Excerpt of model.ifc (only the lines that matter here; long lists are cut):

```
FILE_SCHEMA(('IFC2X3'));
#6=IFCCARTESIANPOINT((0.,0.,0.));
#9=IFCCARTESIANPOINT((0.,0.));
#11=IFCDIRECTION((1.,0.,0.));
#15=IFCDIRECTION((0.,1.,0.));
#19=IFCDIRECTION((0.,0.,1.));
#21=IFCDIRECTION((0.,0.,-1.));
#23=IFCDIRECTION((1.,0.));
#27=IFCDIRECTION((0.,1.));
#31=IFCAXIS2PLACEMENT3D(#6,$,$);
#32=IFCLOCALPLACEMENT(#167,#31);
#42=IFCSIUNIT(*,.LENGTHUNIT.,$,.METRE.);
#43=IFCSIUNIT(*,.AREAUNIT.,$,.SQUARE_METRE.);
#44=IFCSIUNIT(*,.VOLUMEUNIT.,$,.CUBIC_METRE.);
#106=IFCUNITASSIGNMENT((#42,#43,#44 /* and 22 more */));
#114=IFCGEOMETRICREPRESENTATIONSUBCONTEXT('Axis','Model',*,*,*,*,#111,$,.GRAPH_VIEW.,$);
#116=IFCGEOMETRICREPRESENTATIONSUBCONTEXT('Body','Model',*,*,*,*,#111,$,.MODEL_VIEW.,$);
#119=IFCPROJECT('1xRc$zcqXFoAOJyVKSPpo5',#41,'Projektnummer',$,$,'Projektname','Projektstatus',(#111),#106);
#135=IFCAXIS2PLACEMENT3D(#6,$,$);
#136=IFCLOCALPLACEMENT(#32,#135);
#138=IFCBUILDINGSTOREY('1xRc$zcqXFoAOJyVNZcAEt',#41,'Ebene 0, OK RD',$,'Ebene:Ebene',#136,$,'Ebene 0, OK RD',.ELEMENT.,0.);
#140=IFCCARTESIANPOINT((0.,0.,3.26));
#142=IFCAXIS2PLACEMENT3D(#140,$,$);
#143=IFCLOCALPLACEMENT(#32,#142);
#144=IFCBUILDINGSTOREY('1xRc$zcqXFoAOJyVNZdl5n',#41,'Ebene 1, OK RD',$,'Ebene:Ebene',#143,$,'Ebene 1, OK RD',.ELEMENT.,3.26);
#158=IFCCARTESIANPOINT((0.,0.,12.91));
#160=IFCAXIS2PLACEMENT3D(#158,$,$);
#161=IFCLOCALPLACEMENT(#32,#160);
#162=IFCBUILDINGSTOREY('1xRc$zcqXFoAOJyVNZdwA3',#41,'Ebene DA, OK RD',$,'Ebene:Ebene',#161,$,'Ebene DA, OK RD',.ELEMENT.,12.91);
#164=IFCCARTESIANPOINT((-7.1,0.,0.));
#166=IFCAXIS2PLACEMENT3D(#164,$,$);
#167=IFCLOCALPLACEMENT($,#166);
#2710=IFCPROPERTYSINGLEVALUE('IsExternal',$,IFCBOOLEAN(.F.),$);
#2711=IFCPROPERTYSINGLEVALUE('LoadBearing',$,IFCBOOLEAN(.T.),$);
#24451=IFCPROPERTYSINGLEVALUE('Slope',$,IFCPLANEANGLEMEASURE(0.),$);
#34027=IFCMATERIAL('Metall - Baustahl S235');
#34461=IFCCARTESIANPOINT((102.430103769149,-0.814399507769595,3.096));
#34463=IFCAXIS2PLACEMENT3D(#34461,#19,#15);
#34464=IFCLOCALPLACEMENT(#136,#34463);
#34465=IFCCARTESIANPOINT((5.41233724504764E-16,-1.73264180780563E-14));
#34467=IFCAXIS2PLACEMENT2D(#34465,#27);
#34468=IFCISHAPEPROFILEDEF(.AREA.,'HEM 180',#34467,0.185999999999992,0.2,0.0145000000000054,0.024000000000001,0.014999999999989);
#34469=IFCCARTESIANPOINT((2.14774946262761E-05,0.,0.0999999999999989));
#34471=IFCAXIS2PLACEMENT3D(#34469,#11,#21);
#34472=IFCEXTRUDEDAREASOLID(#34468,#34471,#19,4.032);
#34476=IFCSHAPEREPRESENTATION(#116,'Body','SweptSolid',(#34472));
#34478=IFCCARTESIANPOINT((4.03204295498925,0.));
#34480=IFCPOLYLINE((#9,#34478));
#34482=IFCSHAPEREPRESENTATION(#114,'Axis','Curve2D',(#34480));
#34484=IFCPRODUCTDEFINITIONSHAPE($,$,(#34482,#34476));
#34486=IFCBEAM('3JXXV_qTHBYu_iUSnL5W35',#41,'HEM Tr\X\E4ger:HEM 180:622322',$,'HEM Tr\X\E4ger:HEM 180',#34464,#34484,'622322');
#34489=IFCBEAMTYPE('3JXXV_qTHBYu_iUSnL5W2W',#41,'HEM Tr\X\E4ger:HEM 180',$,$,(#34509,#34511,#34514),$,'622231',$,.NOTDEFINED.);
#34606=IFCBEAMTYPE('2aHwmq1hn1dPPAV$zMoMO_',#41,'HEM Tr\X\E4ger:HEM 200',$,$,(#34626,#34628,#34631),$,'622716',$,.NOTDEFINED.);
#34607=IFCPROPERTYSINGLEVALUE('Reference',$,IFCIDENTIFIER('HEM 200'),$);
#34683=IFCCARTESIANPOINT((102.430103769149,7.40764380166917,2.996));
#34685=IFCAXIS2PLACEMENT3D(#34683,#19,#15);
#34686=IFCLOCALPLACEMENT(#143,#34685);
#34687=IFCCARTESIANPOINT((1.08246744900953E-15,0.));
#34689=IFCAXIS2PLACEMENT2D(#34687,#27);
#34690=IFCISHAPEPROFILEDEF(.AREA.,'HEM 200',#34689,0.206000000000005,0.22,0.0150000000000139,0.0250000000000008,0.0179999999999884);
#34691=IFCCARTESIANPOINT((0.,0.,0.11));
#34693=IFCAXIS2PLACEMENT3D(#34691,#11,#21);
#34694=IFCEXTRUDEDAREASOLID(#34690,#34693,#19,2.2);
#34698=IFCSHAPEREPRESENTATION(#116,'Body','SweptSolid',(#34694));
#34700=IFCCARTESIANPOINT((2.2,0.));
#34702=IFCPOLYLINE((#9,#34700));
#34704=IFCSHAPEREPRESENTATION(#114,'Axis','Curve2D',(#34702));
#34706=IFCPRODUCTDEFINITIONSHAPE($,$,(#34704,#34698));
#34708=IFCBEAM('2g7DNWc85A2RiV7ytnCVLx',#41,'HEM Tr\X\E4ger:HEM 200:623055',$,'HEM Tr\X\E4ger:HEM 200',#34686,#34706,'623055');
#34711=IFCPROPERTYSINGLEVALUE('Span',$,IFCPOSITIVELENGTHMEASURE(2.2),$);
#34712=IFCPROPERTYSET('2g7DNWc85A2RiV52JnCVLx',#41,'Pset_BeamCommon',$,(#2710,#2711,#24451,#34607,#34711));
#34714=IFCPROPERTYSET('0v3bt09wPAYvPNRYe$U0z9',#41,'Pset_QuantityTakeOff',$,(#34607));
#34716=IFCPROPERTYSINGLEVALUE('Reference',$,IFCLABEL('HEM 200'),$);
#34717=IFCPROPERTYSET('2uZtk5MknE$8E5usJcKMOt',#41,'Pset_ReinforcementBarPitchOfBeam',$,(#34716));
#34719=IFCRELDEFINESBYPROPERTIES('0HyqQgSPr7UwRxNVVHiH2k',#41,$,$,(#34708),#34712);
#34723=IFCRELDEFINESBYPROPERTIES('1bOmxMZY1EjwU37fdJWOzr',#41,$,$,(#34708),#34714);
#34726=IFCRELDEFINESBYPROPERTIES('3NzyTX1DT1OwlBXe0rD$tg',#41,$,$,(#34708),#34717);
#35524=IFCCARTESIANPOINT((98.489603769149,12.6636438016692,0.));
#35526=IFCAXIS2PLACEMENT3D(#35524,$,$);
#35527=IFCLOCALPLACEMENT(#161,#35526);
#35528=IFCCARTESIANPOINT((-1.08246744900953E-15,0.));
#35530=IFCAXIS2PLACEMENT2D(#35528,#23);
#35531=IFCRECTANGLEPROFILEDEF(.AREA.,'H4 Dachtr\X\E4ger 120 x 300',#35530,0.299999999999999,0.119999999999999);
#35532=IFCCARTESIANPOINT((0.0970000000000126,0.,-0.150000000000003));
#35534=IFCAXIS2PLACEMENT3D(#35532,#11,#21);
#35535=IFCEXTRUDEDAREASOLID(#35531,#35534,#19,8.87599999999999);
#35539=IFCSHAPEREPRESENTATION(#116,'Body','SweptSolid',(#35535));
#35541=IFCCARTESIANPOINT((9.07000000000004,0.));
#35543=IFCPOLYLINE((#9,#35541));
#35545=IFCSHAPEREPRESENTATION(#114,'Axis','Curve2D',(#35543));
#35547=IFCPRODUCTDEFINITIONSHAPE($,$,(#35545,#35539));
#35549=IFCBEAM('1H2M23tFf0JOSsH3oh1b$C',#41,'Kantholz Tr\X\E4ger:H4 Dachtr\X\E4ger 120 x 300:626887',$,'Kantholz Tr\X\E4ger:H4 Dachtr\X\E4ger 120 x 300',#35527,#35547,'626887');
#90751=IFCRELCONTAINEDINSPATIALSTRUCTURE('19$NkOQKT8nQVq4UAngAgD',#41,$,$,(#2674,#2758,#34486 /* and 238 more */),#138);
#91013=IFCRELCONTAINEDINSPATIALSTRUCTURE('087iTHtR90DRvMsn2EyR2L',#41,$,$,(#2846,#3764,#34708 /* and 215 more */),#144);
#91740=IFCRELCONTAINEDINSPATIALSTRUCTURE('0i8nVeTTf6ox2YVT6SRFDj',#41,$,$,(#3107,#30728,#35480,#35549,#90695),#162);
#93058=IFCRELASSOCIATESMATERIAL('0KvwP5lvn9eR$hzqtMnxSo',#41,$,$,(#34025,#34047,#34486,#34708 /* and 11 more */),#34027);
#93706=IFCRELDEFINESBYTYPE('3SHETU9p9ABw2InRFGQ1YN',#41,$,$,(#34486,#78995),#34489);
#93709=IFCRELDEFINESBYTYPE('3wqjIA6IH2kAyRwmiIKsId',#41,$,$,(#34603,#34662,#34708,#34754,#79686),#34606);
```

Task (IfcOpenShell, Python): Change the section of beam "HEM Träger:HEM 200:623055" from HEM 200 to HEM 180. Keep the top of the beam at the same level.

```python
import ifcopenshell
import ifcopenshell.api.pset
import ifcopenshell.api.type
import ifcopenshell.util.element
import ifcopenshell.util.representation

model = ifcopenshell.open("model.ifc")

member = model.by_id(34708)
source = next(p for p in model.by_type("IfcIShapeProfileDef") if p.ProfileName == "HEM 180")

body = ifcopenshell.util.representation.get_representation(member, "Model", "Body")
solid = body.Items[0]
old_profile = solid.SweptArea

# Copy the section's sizes but keep this member's own profile position.
profile = ifcopenshell.util.element.copy(model, source)
# Profiles are centred, so shift by half the change in depth to hold the top.
shift = (old_profile.OverallDepth - profile.OverallDepth) / 2
x, y = old_profile.Position.Location.Coordinates
up = (-1.0, 0.0)  # upwards, in the solid's own plane
location = model.createIfcCartesianPoint((x + up[0] * shift, y + up[1] * shift))
profile.Position = model.createIfcAxis2Placement2D(location, old_profile.Position.RefDirection)
solid.SweptArea = profile
if not model.get_total_inverses(old_profile):
    ifcopenshell.util.element.remove_deep2(model, old_profile)

new_type = model.by_id(34489)
ifcopenshell.api.type.assign_type(
    model, related_objects=[member], relating_type=new_type, should_map_representations=False
)
member.Name = member.Name.replace("HEM 200", "HEM 180")
member.ObjectType = "HEM Träger:HEM 180"
pset = model.by_id(ifcopenshell.util.element.get_pset(member, "Pset_BeamCommon", should_inherit=False)["id"])
ifcopenshell.api.pset.edit_pset(model, pset=pset, properties={"Reference": "HEM 180"})
pset = model.by_id(ifcopenshell.util.element.get_pset(member, "Pset_QuantityTakeOff", should_inherit=False)["id"])
ifcopenshell.api.pset.edit_pset(model, pset=pset, properties={"Reference": "HEM 180"})
pset = model.by_id(ifcopenshell.util.element.get_pset(member, "Pset_ReinforcementBarPitchOfBeam", should_inherit=False)["id"])
ifcopenshell.api.pset.edit_pset(model, pset=pset, properties={"Reference": "HEM 180"})

print(solid.SweptArea)

model.write("model_rev.ifc")
```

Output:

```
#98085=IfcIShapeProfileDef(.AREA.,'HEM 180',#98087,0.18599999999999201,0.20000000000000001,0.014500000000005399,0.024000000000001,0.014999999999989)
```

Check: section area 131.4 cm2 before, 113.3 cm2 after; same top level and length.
